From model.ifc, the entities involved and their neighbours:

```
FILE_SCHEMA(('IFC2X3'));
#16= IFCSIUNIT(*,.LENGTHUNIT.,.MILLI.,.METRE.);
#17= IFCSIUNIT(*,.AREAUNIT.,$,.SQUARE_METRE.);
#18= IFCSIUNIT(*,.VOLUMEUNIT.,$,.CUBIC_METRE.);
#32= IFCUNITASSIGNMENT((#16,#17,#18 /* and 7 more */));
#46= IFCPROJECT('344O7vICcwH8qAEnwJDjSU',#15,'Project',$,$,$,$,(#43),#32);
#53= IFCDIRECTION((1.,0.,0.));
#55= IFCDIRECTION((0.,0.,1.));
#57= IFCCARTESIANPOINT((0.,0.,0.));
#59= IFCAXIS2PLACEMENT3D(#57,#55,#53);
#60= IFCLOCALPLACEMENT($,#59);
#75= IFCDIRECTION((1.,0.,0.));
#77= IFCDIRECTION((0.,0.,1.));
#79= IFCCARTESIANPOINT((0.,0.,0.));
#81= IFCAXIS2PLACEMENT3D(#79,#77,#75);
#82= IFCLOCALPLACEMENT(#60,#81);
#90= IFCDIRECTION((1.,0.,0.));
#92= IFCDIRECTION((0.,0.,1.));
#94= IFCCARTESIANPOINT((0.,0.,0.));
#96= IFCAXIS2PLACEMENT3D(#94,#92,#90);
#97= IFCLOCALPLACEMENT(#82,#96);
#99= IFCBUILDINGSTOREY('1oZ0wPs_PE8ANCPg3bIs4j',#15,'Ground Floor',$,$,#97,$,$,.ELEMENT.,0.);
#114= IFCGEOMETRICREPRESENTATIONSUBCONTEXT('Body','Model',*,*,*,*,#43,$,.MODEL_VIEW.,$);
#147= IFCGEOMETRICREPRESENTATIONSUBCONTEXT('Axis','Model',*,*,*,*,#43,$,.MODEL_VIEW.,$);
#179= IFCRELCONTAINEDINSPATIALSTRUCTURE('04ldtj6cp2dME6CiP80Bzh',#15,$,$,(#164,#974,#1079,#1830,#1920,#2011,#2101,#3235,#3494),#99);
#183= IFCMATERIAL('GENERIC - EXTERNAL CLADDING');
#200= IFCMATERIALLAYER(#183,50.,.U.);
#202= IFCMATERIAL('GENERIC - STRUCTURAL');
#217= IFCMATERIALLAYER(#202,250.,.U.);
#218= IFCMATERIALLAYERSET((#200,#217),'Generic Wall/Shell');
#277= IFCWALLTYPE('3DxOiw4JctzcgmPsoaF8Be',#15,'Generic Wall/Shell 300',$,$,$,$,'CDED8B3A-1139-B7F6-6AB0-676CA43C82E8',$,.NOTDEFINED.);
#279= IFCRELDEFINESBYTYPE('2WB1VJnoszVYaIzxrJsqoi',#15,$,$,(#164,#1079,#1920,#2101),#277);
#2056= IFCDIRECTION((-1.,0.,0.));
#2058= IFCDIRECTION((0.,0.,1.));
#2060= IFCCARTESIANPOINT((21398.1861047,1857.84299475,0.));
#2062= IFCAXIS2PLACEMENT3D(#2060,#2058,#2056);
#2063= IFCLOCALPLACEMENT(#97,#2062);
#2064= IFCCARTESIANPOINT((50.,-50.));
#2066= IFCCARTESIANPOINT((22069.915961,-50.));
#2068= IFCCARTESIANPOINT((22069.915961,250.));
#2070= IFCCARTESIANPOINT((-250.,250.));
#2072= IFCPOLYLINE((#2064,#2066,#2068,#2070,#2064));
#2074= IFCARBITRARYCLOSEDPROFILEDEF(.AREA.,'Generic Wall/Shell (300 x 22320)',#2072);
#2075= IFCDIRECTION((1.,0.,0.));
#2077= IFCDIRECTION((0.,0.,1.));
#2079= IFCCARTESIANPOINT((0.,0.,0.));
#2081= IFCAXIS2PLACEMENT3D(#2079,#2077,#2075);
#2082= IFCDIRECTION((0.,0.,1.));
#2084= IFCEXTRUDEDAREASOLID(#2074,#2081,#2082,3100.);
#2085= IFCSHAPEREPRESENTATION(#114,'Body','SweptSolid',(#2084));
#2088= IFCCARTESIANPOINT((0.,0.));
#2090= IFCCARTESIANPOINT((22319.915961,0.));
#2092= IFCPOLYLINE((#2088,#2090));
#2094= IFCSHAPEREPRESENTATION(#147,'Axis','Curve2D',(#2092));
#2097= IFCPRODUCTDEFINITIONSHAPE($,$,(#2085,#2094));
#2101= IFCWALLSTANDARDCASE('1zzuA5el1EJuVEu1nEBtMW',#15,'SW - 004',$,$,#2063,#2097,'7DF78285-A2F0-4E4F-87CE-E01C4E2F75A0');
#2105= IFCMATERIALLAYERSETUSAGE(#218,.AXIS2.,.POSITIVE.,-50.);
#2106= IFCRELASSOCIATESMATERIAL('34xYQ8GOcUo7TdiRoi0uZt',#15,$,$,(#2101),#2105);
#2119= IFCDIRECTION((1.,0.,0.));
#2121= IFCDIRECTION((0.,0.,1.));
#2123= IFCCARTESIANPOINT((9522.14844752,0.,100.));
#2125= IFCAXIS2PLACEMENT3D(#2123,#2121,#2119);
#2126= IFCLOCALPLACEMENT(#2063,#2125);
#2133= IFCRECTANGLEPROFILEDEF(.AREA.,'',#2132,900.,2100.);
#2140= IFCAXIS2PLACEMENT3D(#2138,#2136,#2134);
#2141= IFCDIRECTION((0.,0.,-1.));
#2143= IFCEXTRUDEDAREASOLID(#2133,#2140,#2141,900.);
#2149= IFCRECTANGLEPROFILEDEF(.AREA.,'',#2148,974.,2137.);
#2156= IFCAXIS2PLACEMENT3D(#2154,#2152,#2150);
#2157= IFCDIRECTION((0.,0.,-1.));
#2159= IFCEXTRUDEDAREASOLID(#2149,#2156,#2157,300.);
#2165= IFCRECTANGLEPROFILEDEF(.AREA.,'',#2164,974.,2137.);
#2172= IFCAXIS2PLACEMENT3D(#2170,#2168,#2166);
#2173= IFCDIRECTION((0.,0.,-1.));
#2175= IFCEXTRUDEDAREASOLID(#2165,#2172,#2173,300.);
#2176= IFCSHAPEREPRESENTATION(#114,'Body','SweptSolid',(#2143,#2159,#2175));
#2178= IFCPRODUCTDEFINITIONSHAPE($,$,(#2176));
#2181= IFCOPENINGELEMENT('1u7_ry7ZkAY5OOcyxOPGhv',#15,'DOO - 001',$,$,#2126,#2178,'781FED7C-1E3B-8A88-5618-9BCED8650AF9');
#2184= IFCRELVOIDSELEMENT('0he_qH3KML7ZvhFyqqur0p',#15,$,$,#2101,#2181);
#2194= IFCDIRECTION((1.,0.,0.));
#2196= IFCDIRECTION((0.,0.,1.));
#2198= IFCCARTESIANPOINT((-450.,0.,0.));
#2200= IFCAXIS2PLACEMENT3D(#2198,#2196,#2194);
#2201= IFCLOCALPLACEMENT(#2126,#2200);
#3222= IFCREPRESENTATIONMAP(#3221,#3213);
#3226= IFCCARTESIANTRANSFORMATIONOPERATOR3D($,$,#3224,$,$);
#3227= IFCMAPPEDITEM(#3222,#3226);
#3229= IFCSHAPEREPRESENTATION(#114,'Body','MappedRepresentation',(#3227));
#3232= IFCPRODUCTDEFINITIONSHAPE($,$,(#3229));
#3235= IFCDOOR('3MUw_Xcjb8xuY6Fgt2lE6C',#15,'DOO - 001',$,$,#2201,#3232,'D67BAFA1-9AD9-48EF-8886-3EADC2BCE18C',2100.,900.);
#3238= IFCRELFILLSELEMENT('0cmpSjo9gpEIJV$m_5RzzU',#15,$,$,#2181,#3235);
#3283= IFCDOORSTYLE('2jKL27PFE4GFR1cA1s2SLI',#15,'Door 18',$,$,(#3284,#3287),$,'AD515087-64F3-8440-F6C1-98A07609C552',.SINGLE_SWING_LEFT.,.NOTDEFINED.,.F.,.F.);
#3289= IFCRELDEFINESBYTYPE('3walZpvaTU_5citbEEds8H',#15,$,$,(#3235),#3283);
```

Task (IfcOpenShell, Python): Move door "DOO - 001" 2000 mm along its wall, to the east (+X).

```python
import ifcopenshell
import ifcopenshell.api.geometry
import ifcopenshell.util.placement

model = ifcopenshell.open("model.ifc")

door = model.by_guid("3MUw_Xcjb8xuY6Fgt2lE6C")
opening = door.FillsVoids[0].RelatingOpeningElement
wall = opening.VoidsElements[0].RelatingBuildingElement

wall_matrix = ifcopenshell.util.placement.get_local_placement(wall.ObjectPlacement)
shift = wall_matrix[:3, 0] * -2000.0
before = ifcopenshell.util.placement.get_local_placement(door.ObjectPlacement)[:3, 3].copy()

# The door is placed relative to its opening, so it follows when the opening moves.
matrix = ifcopenshell.util.placement.get_local_placement(opening.ObjectPlacement)
matrix[:3, 3] += shift
ifcopenshell.api.geometry.edit_object_placement(
    model, product=opening, matrix=matrix, is_si=False, should_transform_children=True
)

after = ifcopenshell.util.placement.get_local_placement(door.ObjectPlacement)[:3, 3]
print("door moved by", (after - before).round(3) + 0.0)

model.write("model_rev.ifc")
```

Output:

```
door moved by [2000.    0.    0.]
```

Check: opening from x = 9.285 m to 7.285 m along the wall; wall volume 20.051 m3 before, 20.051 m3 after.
